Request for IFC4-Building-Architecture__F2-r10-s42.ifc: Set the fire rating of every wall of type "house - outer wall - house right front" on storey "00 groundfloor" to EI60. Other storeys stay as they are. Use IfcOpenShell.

First a look at what the model holds.

```python
import ifcopenshell
import ifcopenshell.util.element

model = ifcopenshell.open("IFC4-Building-Architecture__F2-r10-s42.ifc")
print(model.schema)
storey = next(s for s in model.by_type("IfcBuildingStorey") if s.Name == "00 groundfloor")
walls = [e for e in ifcopenshell.util.element.get_decomposition(storey) if e.is_a("IfcWall")]
seen = {}
for e in walls:
    element_type = ifcopenshell.util.element.get_type(e)
    key = (element_type.Name if element_type != e and element_type else None, ifcopenshell.util.element.get_pset(e, "Pset_WallCommon", "FireRating"))
    seen[key] = seen.get(key, 0) + 1
for (name, value), count in sorted(seen.items(), key=str):
    print(count, "x", name, "|", value)
```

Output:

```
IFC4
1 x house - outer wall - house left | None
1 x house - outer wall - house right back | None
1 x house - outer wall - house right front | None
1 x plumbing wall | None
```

```python
import ifcopenshell
import ifcopenshell.api.pset
import ifcopenshell.util.element

model = ifcopenshell.open("IFC4-Building-Architecture__F2-r10-s42.ifc")

storey = next(s for s in model.by_type("IfcBuildingStorey") if s.Name == "00 groundfloor")
walls = [e for e in ifcopenshell.util.element.get_decomposition(storey) if e.is_a("IfcWall")]

count = 0
for e in walls:
    element_type = ifcopenshell.util.element.get_type(e)
    if element_type in (None, e) or element_type.Name != "house - outer wall - house right front":
        continue
    # add_pset returns the element's existing set when there is one.
    pset = ifcopenshell.api.pset.add_pset(model, product=e, name="Pset_WallCommon")
    ifcopenshell.api.pset.edit_pset(model, pset=pset, properties={"FireRating": "EI60"})
    count += 1

print(count, "walls updated")

model.write("IFC4-Building-Architecture__F2-r10-s42_updated.ifc")
```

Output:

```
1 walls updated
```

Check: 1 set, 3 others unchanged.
